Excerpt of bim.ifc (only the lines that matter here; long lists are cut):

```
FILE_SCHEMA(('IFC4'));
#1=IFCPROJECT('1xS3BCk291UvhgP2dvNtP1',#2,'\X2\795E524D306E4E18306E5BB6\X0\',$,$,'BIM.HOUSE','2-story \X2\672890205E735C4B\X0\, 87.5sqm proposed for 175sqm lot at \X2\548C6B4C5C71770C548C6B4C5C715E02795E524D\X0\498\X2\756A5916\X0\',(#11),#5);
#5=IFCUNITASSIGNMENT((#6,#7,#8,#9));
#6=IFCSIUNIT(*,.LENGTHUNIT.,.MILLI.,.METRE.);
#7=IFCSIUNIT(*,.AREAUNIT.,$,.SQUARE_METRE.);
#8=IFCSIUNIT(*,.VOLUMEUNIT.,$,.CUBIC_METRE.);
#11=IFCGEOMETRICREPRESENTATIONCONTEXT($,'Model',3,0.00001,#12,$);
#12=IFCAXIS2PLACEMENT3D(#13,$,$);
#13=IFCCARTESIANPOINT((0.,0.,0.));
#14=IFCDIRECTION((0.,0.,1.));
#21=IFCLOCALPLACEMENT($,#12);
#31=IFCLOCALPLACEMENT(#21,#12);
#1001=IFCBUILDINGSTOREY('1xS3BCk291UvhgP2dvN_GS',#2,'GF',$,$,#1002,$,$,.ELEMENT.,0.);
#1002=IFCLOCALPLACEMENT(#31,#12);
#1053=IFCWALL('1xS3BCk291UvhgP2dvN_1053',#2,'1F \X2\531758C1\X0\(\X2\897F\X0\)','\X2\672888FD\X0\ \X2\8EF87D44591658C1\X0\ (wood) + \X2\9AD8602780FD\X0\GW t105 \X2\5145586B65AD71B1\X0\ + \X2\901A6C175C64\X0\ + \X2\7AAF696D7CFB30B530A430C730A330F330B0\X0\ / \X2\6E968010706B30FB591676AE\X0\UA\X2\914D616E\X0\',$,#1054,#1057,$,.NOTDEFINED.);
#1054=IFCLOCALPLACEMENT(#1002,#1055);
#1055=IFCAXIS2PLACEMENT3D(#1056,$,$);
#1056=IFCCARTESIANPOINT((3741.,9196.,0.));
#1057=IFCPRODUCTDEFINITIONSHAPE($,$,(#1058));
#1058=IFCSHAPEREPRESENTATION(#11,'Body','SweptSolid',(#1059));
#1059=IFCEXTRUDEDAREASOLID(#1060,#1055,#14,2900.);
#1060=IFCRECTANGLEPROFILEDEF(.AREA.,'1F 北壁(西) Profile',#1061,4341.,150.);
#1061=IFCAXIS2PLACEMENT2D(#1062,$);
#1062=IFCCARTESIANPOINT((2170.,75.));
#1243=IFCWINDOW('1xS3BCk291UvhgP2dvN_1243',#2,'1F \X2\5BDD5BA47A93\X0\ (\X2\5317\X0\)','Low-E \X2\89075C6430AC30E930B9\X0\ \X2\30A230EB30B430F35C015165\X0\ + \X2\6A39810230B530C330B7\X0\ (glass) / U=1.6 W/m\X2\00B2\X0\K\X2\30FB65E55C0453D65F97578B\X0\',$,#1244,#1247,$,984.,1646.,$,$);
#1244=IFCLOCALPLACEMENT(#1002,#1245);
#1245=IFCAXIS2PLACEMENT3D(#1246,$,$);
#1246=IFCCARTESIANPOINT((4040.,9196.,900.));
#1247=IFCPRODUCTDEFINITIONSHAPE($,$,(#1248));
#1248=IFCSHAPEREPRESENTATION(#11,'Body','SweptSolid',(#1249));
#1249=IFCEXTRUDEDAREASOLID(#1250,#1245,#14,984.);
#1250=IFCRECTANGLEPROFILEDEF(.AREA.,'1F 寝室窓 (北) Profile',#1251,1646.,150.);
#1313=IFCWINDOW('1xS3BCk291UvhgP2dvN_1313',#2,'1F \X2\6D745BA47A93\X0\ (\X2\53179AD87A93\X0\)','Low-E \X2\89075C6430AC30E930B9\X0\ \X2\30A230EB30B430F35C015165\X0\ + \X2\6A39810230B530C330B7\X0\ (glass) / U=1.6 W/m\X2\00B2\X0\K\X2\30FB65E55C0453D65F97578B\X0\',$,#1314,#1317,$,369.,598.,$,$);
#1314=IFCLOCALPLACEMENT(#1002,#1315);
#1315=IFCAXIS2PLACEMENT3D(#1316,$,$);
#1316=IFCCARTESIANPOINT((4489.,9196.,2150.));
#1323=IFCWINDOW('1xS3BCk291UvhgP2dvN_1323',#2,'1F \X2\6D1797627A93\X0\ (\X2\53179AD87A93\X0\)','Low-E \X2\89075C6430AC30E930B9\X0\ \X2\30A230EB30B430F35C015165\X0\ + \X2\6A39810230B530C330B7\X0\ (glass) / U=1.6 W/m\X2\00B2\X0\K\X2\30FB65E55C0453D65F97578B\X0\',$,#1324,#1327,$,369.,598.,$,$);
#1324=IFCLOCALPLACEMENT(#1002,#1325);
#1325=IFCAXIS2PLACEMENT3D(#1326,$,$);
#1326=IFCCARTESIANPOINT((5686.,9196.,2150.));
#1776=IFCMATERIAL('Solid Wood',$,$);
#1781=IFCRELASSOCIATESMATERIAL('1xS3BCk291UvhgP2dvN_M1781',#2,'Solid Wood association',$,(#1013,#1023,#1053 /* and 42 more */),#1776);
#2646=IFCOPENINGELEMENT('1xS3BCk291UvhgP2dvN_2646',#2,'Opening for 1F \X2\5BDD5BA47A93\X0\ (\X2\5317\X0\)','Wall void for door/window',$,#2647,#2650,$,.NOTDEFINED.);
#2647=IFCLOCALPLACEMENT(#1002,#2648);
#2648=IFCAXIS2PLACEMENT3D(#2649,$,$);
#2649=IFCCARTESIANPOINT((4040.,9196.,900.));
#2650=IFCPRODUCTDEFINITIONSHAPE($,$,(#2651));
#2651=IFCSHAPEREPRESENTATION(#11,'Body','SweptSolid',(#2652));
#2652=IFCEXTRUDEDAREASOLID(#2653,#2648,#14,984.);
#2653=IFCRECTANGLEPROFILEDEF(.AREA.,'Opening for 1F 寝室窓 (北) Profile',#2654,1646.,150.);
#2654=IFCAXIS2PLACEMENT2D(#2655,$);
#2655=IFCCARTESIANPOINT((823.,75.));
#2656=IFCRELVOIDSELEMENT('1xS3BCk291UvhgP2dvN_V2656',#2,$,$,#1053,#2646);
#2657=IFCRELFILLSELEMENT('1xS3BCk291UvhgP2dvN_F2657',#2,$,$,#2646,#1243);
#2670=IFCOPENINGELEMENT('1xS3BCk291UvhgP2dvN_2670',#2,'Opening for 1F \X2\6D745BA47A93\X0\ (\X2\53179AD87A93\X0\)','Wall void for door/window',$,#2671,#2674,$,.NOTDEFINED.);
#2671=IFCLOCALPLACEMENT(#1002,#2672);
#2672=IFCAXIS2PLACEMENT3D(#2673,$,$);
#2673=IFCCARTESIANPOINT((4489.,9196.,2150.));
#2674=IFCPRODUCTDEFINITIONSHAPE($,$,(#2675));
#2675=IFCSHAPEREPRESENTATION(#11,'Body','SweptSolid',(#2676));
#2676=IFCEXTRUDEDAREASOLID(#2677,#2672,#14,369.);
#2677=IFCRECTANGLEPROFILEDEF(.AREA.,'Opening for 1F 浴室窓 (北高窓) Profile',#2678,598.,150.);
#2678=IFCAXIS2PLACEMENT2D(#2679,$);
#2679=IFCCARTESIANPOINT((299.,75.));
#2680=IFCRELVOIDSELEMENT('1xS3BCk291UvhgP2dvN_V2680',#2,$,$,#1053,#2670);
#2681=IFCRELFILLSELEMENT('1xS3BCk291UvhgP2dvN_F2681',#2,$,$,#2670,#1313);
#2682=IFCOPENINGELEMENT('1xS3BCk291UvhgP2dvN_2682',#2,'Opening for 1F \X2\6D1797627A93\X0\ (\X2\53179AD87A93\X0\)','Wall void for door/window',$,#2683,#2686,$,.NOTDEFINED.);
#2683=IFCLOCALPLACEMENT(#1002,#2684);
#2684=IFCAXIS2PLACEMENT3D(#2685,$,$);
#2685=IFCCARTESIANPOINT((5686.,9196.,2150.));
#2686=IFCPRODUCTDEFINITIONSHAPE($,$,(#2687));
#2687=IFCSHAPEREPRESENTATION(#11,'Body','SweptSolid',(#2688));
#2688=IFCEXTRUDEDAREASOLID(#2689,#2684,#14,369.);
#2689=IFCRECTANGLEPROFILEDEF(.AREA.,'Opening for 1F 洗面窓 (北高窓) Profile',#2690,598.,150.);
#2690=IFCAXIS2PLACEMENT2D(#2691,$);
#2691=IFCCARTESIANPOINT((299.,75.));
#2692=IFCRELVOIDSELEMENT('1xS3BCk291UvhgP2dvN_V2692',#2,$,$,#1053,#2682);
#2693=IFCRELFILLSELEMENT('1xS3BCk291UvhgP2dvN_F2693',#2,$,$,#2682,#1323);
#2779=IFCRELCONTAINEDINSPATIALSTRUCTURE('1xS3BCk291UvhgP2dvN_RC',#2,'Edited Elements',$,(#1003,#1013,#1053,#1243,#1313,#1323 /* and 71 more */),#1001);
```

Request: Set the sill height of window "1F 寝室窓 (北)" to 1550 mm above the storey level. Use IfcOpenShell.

```python
import numpy as np
import ifcopenshell
import ifcopenshell.api.geometry
import ifcopenshell.geom
import ifcopenshell.util.element
import ifcopenshell.util.placement
import ifcopenshell.util.shape
import ifcopenshell.util.unit

model = ifcopenshell.open("bim.ifc")
unit_scale = ifcopenshell.util.unit.calculate_unit_scale(model)

window = model.by_guid("1xS3BCk291UvhgP2dvN_1243")
opening = window.FillsVoids[0].RelatingOpeningElement
storey = ifcopenshell.util.element.get_container(window, ifc_class="IfcBuildingStorey")
level = ifcopenshell.util.placement.get_local_placement(storey.ObjectPlacement)[2, 3]

# The opening's origin need not be at the sill, so measure its lowest point.
shape = ifcopenshell.geom.create_shape(ifcopenshell.geom.settings(), opening)
bottom = ifcopenshell.util.shape.get_shape_bottom_elevation(shape, shape.geometry) / unit_scale
dz = level + 1550.0 - bottom

shift = np.array([0.0, 0.0, dz])
# The window is not placed relative to its opening, so move both.
for product in (opening, window):
    matrix = ifcopenshell.util.placement.get_local_placement(product.ObjectPlacement)
    matrix[:3, 3] += shift
    ifcopenshell.api.geometry.edit_object_placement(model, product=product, matrix=matrix, is_si=False)

print(f"moved by {dz * unit_scale:+.3f} m")

model.write("bim_edited.ifc")
```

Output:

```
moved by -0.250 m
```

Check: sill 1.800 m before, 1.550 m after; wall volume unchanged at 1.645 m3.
